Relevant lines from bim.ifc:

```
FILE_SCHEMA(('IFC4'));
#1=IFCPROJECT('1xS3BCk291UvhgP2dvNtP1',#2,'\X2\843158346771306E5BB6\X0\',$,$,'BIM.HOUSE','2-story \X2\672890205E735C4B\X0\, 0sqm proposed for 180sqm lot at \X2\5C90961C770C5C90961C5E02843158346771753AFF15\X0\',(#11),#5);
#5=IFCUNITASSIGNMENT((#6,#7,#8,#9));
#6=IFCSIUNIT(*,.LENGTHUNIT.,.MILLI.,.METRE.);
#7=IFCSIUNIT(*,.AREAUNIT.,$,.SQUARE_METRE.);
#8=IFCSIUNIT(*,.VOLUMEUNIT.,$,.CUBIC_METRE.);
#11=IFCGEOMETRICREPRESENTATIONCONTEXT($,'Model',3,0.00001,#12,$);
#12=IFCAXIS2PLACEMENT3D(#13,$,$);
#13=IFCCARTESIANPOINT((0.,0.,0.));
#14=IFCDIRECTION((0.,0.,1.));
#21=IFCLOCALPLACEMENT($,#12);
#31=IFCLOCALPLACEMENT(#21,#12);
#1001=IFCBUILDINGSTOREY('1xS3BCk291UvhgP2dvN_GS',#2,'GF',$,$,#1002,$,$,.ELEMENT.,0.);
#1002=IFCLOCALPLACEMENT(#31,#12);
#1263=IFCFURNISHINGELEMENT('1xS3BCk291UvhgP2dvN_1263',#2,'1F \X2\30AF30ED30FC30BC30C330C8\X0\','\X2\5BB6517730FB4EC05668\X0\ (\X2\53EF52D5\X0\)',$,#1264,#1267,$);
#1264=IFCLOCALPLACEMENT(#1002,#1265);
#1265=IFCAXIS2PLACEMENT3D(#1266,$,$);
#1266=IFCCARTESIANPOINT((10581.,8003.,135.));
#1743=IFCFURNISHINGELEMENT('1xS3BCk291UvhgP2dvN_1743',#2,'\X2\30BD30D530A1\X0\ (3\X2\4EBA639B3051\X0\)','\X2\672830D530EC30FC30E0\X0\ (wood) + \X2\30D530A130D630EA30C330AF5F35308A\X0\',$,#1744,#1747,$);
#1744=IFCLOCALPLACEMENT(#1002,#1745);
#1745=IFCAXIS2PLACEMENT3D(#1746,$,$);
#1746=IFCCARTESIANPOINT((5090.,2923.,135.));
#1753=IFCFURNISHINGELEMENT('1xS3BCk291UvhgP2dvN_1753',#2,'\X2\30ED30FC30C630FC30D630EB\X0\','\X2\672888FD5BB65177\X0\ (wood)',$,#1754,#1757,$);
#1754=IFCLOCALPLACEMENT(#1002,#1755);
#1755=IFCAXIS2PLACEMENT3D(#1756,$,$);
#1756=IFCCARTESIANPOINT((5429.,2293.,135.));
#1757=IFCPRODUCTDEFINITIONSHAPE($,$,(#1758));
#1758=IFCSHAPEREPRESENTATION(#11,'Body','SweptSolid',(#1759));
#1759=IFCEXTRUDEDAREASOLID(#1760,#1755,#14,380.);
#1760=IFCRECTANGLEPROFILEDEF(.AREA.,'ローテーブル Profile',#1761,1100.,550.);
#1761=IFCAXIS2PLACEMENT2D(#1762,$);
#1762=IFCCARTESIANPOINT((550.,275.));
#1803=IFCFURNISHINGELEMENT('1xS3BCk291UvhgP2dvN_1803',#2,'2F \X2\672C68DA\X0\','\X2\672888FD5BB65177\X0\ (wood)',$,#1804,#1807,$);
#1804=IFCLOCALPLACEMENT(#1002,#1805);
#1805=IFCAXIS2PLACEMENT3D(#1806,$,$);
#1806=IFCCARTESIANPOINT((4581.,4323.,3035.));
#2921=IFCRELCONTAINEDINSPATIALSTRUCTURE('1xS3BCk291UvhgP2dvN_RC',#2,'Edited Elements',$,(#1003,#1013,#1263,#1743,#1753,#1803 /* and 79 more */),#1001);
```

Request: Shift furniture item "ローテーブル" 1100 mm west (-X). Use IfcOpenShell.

```python
import ifcopenshell
import ifcopenshell.api.geometry
import ifcopenshell.util.placement

model = ifcopenshell.open("bim.ifc")

item = model.by_guid("1xS3BCk291UvhgP2dvN_1753")
matrix = ifcopenshell.util.placement.get_local_placement(item.ObjectPlacement)
matrix[0, 3] -= 1100.0
ifcopenshell.api.geometry.edit_object_placement(model, product=item, matrix=matrix, is_si=False)

print(ifcopenshell.util.placement.get_local_placement(item.ObjectPlacement).round(3) + 0.0)

model.write("bim_v2.ifc")
```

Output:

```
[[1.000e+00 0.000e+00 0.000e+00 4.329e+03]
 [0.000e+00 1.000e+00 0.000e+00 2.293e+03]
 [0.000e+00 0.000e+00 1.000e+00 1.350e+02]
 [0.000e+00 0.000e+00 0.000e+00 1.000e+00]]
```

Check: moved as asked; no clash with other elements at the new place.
